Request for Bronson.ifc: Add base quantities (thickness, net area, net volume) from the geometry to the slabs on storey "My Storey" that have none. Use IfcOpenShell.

First a look at what the model holds.

```python
import ifcopenshell
import ifcopenshell.util.element
import ifcopenshell.util.unit

model = ifcopenshell.open("Bronson.ifc")
print(model.schema)
for unit_type in ("LENGTHUNIT", "AREAUNIT", "VOLUMEUNIT"):
    print(unit_type, ifcopenshell.util.unit.calculate_unit_scale(model, unit_type))
storey = next(s for s in model.by_type("IfcBuildingStorey") if s.Name == "My Storey")
slabs = [e for e in ifcopenshell.util.element.get_decomposition(storey) if e.is_a("IfcSlab")]
for e in sorted(slabs, key=lambda e: e.id()):
    print(e.id(), e.is_a(), e.Name, list(ifcopenshell.util.element.get_psets(e, qtos_only=True)), sep=" | ")
```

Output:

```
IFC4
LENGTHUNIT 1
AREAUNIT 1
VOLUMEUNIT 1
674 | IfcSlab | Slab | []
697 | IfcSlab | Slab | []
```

```python
import ifcopenshell
import ifcopenshell.api.pset
import ifcopenshell.geom
import ifcopenshell.util.element
import ifcopenshell.util.shape
import ifcopenshell.util.unit

model = ifcopenshell.open("Bronson.ifc")
unit_scale = ifcopenshell.util.unit.calculate_unit_scale(model)
area_scale = ifcopenshell.util.unit.calculate_unit_scale(model, "AREAUNIT")
volume_scale = ifcopenshell.util.unit.calculate_unit_scale(model, "VOLUMEUNIT")
settings = ifcopenshell.geom.settings()

storey = next(s for s in model.by_type("IfcBuildingStorey") if s.Name == "My Storey")
slabs = [e for e in ifcopenshell.util.element.get_decomposition(storey) if e.is_a("IfcSlab")]

for e in sorted(slabs, key=lambda e: e.id()):
    if ifcopenshell.util.element.get_psets(e, qtos_only=True, should_inherit=False):
        continue
    # Geometry comes back in metres, in the element's own axes.
    shape = ifcopenshell.geom.create_shape(settings, e)
    values = {
        "Width": ifcopenshell.util.shape.get_z(shape.geometry) / unit_scale,
        "NetArea": ifcopenshell.util.shape.get_footprint_area(shape.geometry) / area_scale,
        "NetVolume": ifcopenshell.util.shape.get_volume(shape.geometry) / volume_scale,
    }
    qto = ifcopenshell.api.pset.add_qto(model, product=e, name="Qto_SlabBaseQuantities")
    ifcopenshell.api.pset.edit_qto(model, qto=qto, properties=values)
    print(e.id(), {k: round(v, 3) for k, v in values.items()})

model.write("Bronson_rev.ifc")
```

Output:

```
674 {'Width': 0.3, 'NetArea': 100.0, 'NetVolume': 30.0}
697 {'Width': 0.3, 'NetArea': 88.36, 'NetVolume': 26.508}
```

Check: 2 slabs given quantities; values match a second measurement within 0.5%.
